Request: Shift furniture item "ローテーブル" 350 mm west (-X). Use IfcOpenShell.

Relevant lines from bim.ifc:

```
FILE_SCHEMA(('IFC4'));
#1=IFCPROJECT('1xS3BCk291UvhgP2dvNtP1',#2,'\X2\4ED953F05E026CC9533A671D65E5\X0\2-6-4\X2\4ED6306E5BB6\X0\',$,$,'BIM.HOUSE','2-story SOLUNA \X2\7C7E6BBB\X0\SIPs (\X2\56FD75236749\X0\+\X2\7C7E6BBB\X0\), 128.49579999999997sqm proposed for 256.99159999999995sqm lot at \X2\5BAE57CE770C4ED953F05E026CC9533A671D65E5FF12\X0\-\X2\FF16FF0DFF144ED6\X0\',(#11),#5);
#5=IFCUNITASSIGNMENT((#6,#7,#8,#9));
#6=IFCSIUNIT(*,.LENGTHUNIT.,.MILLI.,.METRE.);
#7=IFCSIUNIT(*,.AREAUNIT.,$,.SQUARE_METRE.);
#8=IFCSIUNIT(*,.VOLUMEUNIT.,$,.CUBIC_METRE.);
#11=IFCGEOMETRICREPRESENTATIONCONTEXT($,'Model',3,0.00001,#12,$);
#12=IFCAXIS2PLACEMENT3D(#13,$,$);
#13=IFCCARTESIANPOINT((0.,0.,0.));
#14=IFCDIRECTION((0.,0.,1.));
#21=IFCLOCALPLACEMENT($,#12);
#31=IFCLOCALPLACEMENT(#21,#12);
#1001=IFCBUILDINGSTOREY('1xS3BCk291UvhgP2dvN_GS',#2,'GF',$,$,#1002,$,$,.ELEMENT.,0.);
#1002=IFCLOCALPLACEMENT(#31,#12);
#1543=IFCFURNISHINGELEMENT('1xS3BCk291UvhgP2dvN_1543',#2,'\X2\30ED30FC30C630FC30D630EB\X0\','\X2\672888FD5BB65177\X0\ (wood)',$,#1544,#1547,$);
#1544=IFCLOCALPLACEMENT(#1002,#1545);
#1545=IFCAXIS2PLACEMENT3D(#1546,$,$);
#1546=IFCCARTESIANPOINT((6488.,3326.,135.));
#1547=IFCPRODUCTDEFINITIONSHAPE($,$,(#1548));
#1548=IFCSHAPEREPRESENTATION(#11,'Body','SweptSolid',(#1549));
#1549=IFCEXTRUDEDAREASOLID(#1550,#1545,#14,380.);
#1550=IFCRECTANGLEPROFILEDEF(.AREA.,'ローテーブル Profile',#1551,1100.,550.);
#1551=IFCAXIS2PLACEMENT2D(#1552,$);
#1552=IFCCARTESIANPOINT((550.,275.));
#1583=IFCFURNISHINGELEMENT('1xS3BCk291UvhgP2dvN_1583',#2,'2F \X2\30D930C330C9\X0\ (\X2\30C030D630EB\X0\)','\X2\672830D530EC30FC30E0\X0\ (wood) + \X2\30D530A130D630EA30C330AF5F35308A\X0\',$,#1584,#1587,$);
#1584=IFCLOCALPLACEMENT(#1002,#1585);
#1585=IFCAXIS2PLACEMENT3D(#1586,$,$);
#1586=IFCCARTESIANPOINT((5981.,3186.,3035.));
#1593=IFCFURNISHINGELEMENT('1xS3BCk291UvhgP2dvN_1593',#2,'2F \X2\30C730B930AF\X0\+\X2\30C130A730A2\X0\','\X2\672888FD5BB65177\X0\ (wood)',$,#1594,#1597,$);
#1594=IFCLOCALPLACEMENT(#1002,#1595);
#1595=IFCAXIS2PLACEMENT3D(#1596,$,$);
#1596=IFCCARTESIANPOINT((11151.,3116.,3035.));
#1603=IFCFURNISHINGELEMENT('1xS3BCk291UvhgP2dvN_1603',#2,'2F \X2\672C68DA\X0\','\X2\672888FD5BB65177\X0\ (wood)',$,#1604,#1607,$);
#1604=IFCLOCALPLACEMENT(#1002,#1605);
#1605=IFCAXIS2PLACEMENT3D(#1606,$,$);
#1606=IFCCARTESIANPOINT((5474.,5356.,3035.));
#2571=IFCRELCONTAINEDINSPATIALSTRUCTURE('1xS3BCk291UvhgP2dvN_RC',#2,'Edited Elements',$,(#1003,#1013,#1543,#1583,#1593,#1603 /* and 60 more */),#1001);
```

```python
import ifcopenshell
import ifcopenshell.api.geometry
import ifcopenshell.util.placement
import ifcopenshell.util.unit

model = ifcopenshell.open("bim.ifc")
unit_scale = ifcopenshell.util.unit.calculate_unit_scale(model)

item = model.by_id(1543)
matrix = ifcopenshell.util.placement.get_local_placement(item.ObjectPlacement)
matrix[0, 3] -= 0.35 / unit_scale
ifcopenshell.api.geometry.edit_object_placement(model, product=item, matrix=matrix, is_si=False)

print(ifcopenshell.util.placement.get_local_placement(item.ObjectPlacement).round(3) + 0.0)

model.write("bim_edited.ifc")
```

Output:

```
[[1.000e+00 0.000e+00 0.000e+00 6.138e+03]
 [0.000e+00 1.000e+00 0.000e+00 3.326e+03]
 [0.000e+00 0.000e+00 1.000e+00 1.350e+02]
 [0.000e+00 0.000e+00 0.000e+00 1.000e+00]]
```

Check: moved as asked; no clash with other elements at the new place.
